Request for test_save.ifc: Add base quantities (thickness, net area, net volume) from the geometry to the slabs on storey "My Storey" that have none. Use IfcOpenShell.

First a look at what the model holds.

```python
import ifcopenshell
import ifcopenshell.util.element
import ifcopenshell.util.unit

model = ifcopenshell.open("test_save.ifc")
print(model.schema)
for unit_type in ("LENGTHUNIT", "AREAUNIT", "VOLUMEUNIT"):
    print(unit_type, ifcopenshell.util.unit.calculate_unit_scale(model, unit_type))
storey = next(s for s in model.by_type("IfcBuildingStorey") if s.Name == "My Storey")
slabs = [e for e in ifcopenshell.util.element.get_decomposition(storey) if e.is_a("IfcSlab")]
for e in sorted(slabs, key=lambda e: e.id()):
    print(e.id(), e.is_a(), e.Name, list(ifcopenshell.util.element.get_psets(e, qtos_only=True)), sep=" | ")
```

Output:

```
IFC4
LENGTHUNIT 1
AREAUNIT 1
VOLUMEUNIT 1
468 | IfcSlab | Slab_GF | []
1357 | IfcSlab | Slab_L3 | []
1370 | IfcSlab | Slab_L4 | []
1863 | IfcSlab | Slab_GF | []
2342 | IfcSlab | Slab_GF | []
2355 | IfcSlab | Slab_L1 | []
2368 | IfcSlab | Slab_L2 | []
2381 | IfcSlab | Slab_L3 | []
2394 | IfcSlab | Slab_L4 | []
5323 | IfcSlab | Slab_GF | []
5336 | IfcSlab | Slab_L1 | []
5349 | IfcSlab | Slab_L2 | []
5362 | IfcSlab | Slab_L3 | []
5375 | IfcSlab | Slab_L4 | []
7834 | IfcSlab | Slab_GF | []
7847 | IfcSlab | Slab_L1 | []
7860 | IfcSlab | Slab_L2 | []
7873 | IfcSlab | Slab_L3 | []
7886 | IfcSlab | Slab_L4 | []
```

```python
import ifcopenshell
import ifcopenshell.api.pset
import ifcopenshell.geom
import ifcopenshell.util.element
import ifcopenshell.util.shape
import ifcopenshell.util.unit

model = ifcopenshell.open("test_save.ifc")
unit_scale = ifcopenshell.util.unit.calculate_unit_scale(model)
area_scale = ifcopenshell.util.unit.calculate_unit_scale(model, "AREAUNIT")
volume_scale = ifcopenshell.util.unit.calculate_unit_scale(model, "VOLUMEUNIT")
settings = ifcopenshell.geom.settings()

storey = next(s for s in model.by_type("IfcBuildingStorey") if s.Name == "My Storey")
slabs = [e for e in ifcopenshell.util.element.get_decomposition(storey) if e.is_a("IfcSlab")]

for e in sorted(slabs, key=lambda e: e.id()):
    if ifcopenshell.util.element.get_psets(e, qtos_only=True, should_inherit=False):
        continue
    # Geometry comes back in metres, in the element's own axes.
    shape = ifcopenshell.geom.create_shape(settings, e)
    values = {
        "Width": ifcopenshell.util.shape.get_z(shape.geometry) / unit_scale,
        "NetArea": ifcopenshell.util.shape.get_footprint_area(shape.geometry) / area_scale,
        "NetVolume": ifcopenshell.util.shape.get_volume(shape.geometry) / volume_scale,
    }
    qto = ifcopenshell.api.pset.add_qto(model, product=e, name="Qto_SlabBaseQuantities")
    ifcopenshell.api.pset.edit_qto(model, qto=qto, properties=values)
    print(e.id(), {k: round(v, 3) for k, v in values.items()})

model.write("test_save_rev.ifc")
```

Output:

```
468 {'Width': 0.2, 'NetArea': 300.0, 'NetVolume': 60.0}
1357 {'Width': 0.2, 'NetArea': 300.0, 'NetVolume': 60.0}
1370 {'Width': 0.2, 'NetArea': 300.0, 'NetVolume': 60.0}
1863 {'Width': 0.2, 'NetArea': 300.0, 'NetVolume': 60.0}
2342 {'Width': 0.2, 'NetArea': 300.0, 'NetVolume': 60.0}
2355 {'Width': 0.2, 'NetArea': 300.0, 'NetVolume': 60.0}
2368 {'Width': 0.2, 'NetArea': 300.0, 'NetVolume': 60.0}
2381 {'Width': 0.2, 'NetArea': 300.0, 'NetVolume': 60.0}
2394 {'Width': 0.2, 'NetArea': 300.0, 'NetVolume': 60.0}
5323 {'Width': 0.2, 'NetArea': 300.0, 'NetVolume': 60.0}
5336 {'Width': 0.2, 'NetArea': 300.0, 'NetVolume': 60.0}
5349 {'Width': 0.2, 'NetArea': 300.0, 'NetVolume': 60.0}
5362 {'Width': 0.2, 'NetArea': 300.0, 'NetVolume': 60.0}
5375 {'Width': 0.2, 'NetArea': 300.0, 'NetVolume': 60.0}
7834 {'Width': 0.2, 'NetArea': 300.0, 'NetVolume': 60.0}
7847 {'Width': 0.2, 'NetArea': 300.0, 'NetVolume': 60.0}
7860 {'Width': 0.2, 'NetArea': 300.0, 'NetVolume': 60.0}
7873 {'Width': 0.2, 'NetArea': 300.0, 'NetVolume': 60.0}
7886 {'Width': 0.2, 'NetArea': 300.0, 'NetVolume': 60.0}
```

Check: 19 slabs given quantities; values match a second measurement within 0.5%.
